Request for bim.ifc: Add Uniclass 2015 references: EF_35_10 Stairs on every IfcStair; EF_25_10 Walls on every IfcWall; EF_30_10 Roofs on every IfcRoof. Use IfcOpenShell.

First a look at what the model holds.

```python
import ifcopenshell

model = ifcopenshell.open("bim.ifc")
print(model.schema)
print("classifications:", [c.Name for c in model.by_type("IfcClassification")])
for ifc_class in ("IfcDoor", "IfcRoof", "IfcStair", "IfcWall", "IfcWindow"):
    print(ifc_class, len(model.by_type(ifc_class)))
```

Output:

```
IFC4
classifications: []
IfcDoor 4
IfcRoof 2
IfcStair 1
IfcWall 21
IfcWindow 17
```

```python
import ifcopenshell
import ifcopenshell.api.classification

model = ifcopenshell.open("bim.ifc")

system = ifcopenshell.api.classification.add_classification(model, classification="Uniclass 2015")

codes = {
    "IfcStair": ("EF_35_10", "Stairs"),
    "IfcWall": ("EF_25_10", "Walls"),
    "IfcRoof": ("EF_30_10", "Roofs"),
}
for ifc_class, (code, name) in codes.items():
    products = model.by_type(ifc_class)
    ifcopenshell.api.classification.add_reference(
        model, products=products, classification=system, identification=code, name=name
    )
    print(code, len(products))

model.write("bim_v2.ifc")
```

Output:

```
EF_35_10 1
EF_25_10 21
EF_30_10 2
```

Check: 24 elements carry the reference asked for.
